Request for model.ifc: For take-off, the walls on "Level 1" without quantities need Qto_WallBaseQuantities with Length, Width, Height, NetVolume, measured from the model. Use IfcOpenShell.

First a look at what the model holds.

```python
import ifcopenshell
import ifcopenshell.util.element
import ifcopenshell.util.unit

model = ifcopenshell.open("model.ifc")
print(model.schema)
for unit_type in ("LENGTHUNIT", "AREAUNIT", "VOLUMEUNIT"):
    print(unit_type, ifcopenshell.util.unit.calculate_unit_scale(model, unit_type))
storey = next(s for s in model.by_type("IfcBuildingStorey") if s.Name == "Level 1")
walls = [e for e in ifcopenshell.util.element.get_decomposition(storey) if e.is_a("IfcWall")]
for e in sorted(walls, key=lambda e: e.id()):
    print(e.id(), e.is_a(), e.Name, list(ifcopenshell.util.element.get_psets(e, qtos_only=True)), sep=" | ")
```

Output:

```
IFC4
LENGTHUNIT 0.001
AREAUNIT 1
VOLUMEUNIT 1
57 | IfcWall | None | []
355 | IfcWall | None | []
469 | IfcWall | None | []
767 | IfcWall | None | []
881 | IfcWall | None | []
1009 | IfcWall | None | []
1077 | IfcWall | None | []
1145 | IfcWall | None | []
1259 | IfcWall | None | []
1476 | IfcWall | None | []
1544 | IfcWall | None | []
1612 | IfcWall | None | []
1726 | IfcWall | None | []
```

```python
import ifcopenshell
import ifcopenshell.api.pset
import ifcopenshell.geom
import ifcopenshell.util.element
import ifcopenshell.util.shape
import ifcopenshell.util.unit

model = ifcopenshell.open("model.ifc")
unit_scale = ifcopenshell.util.unit.calculate_unit_scale(model)
volume_scale = ifcopenshell.util.unit.calculate_unit_scale(model, "VOLUMEUNIT")
settings = ifcopenshell.geom.settings()

storey = next(s for s in model.by_type("IfcBuildingStorey") if s.Name == "Level 1")
walls = [e for e in ifcopenshell.util.element.get_decomposition(storey) if e.is_a("IfcWall")]

for e in sorted(walls, key=lambda e: e.id()):
    if ifcopenshell.util.element.get_psets(e, qtos_only=True, should_inherit=False):
        continue
    # Geometry comes back in metres, in the element's own axes.
    shape = ifcopenshell.geom.create_shape(settings, e)
    values = {
        "Length": ifcopenshell.util.shape.get_x(shape.geometry) / unit_scale,
        "Width": ifcopenshell.util.shape.get_y(shape.geometry) / unit_scale,
        "Height": ifcopenshell.util.shape.get_z(shape.geometry) / unit_scale,
        "NetVolume": ifcopenshell.util.shape.get_volume(shape.geometry) / volume_scale,
    }
    qto = ifcopenshell.api.pset.add_qto(model, product=e, name="Qto_WallBaseQuantities")
    ifcopenshell.api.pset.edit_qto(model, qto=qto, properties=values)
    print(e.id(), {k: round(v, 3) for k, v in values.items()})

model.write("model_v2.ifc")
```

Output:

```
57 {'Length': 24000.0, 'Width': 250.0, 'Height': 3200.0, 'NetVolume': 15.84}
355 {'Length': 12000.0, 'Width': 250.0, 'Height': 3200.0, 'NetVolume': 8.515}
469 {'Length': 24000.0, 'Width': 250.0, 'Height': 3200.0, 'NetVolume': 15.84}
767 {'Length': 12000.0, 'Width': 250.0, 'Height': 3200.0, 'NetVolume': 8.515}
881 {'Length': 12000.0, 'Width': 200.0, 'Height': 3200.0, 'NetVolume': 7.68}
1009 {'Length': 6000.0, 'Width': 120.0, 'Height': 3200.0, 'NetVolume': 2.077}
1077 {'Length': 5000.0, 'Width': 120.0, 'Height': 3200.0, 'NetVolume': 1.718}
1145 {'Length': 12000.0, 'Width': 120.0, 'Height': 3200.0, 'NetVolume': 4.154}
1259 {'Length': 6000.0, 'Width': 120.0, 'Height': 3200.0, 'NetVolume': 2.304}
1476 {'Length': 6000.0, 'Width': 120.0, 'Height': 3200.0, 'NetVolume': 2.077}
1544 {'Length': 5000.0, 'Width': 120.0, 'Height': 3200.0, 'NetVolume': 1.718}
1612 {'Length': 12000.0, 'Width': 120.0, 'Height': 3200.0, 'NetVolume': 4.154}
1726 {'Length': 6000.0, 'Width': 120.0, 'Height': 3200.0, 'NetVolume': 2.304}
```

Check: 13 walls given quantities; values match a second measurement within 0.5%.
